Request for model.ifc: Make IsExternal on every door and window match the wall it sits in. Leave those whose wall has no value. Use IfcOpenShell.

First a look at what the model holds.

```python
import ifcopenshell
import ifcopenshell.util.element

model = ifcopenshell.open("model.ifc")
print(model.schema)
seen = {}
for e in model.by_type("IfcDoor") + model.by_type("IfcWindow"):
    if not e.FillsVoids:
        continue
    host = e.FillsVoids[0].RelatingOpeningElement.VoidsElements[0].RelatingBuildingElement
    own = ifcopenshell.util.element.get_pset(e, f"Pset_{e.is_a()[3:].removesuffix('StandardCase')}Common", "IsExternal")
    wall = ifcopenshell.util.element.get_pset(host, "Pset_WallCommon", "IsExternal")
    seen[e.is_a(), own, wall] = seen.get((e.is_a(), own, wall), 0) + 1
for (cls, own, wall), count in sorted(seen.items(), key=str):
    print(count, cls, "IsExternal:", own, "| host wall:", wall)
```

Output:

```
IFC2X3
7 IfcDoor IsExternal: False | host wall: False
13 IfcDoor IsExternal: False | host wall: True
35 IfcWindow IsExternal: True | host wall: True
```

```python
import ifcopenshell
import ifcopenshell.api.pset
import ifcopenshell.util.element

model = ifcopenshell.open("model.ifc")

count = 0
for ifc_class, pset_name in (("IfcDoor", "Pset_DoorCommon"), ("IfcWindow", "Pset_WindowCommon")):
    for e in model.by_type(ifc_class):
        if not e.FillsVoids:
            continue
        host = e.FillsVoids[0].RelatingOpeningElement.VoidsElements[0].RelatingBuildingElement
        external = ifcopenshell.util.element.get_pset(host, "Pset_WallCommon", "IsExternal")
        if external is None or ifcopenshell.util.element.get_pset(e, pset_name, "IsExternal") == external:
            continue
        pset = ifcopenshell.api.pset.add_pset(model, product=e, name=pset_name)
        ifcopenshell.api.pset.edit_pset(model, pset=pset, properties={"IsExternal": external})
        count += 1

print(count, "updated")

model.write("model-out.ifc")
```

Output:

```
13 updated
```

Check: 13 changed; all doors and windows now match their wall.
